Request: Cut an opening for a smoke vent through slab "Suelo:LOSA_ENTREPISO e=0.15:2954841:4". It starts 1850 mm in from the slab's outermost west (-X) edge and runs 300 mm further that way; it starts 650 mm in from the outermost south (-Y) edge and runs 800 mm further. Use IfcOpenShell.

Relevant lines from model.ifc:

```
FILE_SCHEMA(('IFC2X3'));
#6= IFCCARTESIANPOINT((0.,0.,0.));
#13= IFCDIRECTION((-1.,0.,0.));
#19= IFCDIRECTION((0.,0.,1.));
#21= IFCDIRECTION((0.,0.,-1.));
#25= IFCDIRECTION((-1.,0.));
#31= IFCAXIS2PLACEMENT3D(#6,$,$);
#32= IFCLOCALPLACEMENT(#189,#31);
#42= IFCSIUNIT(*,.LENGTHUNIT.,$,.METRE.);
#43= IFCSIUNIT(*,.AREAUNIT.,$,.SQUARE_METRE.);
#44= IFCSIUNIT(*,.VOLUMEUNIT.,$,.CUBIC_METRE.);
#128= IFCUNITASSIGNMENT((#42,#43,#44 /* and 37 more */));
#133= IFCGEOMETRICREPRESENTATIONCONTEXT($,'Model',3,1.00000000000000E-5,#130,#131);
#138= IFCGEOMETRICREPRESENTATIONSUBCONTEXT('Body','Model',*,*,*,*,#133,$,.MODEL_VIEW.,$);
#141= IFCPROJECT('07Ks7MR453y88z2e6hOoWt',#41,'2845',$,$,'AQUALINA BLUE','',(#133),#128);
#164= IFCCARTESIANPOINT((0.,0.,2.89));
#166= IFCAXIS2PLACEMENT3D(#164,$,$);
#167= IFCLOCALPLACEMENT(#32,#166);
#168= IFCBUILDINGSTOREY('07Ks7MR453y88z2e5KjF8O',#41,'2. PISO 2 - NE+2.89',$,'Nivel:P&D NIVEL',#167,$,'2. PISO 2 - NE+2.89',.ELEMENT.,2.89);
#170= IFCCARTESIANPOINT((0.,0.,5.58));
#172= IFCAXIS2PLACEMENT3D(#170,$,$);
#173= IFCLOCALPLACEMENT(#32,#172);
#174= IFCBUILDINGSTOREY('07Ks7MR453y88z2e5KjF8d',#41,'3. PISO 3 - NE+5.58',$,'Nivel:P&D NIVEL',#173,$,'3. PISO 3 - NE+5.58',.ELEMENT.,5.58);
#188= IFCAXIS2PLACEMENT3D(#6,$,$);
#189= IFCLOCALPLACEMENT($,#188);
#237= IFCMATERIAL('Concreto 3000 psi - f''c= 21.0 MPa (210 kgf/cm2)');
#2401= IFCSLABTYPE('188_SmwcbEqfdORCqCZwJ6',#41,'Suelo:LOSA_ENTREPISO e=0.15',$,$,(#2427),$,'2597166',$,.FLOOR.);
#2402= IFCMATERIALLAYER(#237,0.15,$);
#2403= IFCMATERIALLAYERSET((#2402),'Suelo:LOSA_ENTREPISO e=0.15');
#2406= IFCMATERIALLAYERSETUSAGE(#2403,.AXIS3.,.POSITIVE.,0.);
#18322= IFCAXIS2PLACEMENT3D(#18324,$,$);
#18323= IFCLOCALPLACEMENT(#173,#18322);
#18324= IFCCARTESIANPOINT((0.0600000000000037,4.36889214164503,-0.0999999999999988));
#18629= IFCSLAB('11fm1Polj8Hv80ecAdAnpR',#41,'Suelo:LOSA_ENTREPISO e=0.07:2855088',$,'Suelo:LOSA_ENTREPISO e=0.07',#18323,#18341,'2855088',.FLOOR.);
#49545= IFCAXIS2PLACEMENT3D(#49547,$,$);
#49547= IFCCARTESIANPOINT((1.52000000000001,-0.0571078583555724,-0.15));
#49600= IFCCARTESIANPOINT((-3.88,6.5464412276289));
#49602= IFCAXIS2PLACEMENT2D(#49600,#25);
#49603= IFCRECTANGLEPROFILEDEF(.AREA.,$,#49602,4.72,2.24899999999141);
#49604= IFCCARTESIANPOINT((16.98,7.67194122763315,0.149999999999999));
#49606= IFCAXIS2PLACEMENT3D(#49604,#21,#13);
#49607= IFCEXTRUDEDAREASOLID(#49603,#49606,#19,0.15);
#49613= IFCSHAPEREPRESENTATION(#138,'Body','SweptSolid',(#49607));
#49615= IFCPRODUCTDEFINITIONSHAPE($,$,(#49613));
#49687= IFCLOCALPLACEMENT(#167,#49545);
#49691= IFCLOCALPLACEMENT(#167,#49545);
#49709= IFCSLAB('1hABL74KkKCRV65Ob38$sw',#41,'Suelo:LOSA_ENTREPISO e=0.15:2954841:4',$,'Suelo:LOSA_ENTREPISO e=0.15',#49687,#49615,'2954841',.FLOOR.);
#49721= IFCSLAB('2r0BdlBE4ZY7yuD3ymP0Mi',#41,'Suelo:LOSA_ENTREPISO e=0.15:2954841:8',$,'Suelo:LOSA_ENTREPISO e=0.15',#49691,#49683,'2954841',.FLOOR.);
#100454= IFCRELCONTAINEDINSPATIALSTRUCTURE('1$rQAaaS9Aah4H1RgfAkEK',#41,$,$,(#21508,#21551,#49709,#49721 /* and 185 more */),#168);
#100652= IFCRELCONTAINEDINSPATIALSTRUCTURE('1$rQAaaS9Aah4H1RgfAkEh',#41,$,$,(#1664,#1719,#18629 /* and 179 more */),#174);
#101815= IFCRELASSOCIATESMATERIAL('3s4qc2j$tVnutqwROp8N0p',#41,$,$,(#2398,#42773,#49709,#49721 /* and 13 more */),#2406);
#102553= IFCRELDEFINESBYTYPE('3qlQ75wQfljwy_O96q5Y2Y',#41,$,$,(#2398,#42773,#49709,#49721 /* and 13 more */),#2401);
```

```python
import numpy as np
import ifcopenshell
import ifcopenshell.api.feature
import ifcopenshell.api.geometry
import ifcopenshell.api.root
import ifcopenshell.geom
import ifcopenshell.util.placement
import ifcopenshell.util.representation
import ifcopenshell.util.shape
import ifcopenshell.util.unit

model = ifcopenshell.open("model.ifc")
unit_scale = ifcopenshell.util.unit.calculate_unit_scale(model)
settings = ifcopenshell.geom.settings()


def volume(element):
    """Net volume in cubic metres, openings subtracted."""
    shape = ifcopenshell.geom.create_shape(settings, element)
    return ifcopenshell.util.shape.get_volume(shape.geometry)


slab = model.by_id(49709)
before = volume(slab)

# Extent in the slab's own axes, in metres. The edges named are its -X and -Y sides.
slab_shape = ifcopenshell.geom.create_shape(settings, slab)
vertices = ifcopenshell.util.shape.get_vertices(slab_shape.geometry)
x_min, y_min, bottom = vertices.min(axis=0)
top = vertices[:, 2].max()

opening = ifcopenshell.api.root.create_entity(model, ifc_class="IfcOpeningElement", name="Smoke vent opening")
context = ifcopenshell.util.representation.get_context(model, "Model", "Body", "MODEL_VIEW")
width, depth = 0.3, 0.8
outline = [(0.0, 0.0), (width, 0.0), (width, depth), (0.0, depth), (0.0, 0.0)]
# Overshoot both faces by 50 mm so the cut is clean.
shape = ifcopenshell.api.geometry.add_slab_representation(
    model, context=context, depth=top - bottom + 0.1, polyline=outline
)
ifcopenshell.api.geometry.assign_representation(model, product=opening, representation=shape)

matrix = ifcopenshell.util.placement.get_local_placement(slab.ObjectPlacement)
matrix[:, 3] = matrix @ np.append(np.array([x_min + 1.85, y_min + 0.65, bottom - 0.05]) / unit_scale, 1.0)
ifcopenshell.api.geometry.edit_object_placement(model, product=opening, matrix=matrix, is_si=False)
ifcopenshell.api.feature.add_feature(model, feature=opening, element=slab)

after = volume(slab)

print(f"slab volume {before:.3f} -> {after:.3f} m3")

model.write("model_updated.ifc")
```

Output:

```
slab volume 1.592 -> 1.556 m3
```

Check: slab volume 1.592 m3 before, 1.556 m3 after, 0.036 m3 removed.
